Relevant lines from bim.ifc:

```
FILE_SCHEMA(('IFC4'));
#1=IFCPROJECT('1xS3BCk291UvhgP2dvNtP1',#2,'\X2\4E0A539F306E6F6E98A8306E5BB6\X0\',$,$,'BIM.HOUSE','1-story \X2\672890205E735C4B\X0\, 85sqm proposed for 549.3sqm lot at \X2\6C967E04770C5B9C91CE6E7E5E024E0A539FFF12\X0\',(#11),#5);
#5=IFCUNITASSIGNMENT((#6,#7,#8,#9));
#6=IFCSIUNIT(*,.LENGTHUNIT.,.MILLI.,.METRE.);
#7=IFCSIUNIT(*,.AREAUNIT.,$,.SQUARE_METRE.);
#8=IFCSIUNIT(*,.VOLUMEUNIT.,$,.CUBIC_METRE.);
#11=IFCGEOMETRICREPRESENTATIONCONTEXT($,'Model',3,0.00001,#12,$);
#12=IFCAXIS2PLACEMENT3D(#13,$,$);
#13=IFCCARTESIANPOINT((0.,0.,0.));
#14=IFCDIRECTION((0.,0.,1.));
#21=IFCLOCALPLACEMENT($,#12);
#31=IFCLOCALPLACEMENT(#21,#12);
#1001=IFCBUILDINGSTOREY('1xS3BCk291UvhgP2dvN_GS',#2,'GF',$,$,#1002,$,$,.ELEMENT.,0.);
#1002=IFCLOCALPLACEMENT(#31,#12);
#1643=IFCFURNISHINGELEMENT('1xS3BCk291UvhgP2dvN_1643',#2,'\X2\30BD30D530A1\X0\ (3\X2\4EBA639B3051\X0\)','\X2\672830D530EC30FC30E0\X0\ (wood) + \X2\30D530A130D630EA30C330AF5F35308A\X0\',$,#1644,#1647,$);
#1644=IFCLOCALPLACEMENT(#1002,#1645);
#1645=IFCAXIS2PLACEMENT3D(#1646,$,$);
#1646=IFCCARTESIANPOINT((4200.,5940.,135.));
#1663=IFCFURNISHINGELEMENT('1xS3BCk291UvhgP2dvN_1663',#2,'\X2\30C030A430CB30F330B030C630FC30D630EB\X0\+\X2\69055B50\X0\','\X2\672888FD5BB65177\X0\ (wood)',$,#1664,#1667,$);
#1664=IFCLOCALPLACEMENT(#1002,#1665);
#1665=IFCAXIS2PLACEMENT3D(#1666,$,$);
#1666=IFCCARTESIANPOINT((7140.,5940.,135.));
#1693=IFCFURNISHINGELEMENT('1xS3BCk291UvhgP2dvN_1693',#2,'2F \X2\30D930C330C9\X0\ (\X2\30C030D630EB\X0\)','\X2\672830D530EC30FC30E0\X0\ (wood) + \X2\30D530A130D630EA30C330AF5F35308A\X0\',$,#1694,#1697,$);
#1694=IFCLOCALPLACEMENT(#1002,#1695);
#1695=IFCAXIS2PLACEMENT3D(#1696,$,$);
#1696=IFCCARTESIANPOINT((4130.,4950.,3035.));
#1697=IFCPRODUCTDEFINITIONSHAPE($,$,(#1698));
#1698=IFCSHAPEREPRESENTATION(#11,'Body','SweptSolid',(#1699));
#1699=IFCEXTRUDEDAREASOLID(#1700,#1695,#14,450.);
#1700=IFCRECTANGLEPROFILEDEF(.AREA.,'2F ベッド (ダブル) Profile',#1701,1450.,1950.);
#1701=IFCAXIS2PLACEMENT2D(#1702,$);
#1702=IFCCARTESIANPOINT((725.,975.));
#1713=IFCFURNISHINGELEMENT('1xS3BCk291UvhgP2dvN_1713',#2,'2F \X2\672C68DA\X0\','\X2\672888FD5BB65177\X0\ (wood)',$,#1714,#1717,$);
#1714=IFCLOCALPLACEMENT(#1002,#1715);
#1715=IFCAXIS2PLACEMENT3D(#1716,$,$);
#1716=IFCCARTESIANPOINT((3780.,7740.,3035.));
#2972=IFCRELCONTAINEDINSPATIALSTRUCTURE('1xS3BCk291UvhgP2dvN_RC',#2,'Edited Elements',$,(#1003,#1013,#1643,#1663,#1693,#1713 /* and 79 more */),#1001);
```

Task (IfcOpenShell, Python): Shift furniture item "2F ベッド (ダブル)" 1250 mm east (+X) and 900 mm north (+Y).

```python
import ifcopenshell
import ifcopenshell.api.geometry
import ifcopenshell.util.placement

model = ifcopenshell.open("bim.ifc")

item = model.by_guid("1xS3BCk291UvhgP2dvN_1693")
matrix = ifcopenshell.util.placement.get_local_placement(item.ObjectPlacement)
matrix[0, 3] += 1250.0
matrix[1, 3] += 900.0
ifcopenshell.api.geometry.edit_object_placement(model, product=item, matrix=matrix, is_si=False)

print(ifcopenshell.util.placement.get_local_placement(item.ObjectPlacement).round(3) + 0.0)

model.write("bim_updated.ifc")
```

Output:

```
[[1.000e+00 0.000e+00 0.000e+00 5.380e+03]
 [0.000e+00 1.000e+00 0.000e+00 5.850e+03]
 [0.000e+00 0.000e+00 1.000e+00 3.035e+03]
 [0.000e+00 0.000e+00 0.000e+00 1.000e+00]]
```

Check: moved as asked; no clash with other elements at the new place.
